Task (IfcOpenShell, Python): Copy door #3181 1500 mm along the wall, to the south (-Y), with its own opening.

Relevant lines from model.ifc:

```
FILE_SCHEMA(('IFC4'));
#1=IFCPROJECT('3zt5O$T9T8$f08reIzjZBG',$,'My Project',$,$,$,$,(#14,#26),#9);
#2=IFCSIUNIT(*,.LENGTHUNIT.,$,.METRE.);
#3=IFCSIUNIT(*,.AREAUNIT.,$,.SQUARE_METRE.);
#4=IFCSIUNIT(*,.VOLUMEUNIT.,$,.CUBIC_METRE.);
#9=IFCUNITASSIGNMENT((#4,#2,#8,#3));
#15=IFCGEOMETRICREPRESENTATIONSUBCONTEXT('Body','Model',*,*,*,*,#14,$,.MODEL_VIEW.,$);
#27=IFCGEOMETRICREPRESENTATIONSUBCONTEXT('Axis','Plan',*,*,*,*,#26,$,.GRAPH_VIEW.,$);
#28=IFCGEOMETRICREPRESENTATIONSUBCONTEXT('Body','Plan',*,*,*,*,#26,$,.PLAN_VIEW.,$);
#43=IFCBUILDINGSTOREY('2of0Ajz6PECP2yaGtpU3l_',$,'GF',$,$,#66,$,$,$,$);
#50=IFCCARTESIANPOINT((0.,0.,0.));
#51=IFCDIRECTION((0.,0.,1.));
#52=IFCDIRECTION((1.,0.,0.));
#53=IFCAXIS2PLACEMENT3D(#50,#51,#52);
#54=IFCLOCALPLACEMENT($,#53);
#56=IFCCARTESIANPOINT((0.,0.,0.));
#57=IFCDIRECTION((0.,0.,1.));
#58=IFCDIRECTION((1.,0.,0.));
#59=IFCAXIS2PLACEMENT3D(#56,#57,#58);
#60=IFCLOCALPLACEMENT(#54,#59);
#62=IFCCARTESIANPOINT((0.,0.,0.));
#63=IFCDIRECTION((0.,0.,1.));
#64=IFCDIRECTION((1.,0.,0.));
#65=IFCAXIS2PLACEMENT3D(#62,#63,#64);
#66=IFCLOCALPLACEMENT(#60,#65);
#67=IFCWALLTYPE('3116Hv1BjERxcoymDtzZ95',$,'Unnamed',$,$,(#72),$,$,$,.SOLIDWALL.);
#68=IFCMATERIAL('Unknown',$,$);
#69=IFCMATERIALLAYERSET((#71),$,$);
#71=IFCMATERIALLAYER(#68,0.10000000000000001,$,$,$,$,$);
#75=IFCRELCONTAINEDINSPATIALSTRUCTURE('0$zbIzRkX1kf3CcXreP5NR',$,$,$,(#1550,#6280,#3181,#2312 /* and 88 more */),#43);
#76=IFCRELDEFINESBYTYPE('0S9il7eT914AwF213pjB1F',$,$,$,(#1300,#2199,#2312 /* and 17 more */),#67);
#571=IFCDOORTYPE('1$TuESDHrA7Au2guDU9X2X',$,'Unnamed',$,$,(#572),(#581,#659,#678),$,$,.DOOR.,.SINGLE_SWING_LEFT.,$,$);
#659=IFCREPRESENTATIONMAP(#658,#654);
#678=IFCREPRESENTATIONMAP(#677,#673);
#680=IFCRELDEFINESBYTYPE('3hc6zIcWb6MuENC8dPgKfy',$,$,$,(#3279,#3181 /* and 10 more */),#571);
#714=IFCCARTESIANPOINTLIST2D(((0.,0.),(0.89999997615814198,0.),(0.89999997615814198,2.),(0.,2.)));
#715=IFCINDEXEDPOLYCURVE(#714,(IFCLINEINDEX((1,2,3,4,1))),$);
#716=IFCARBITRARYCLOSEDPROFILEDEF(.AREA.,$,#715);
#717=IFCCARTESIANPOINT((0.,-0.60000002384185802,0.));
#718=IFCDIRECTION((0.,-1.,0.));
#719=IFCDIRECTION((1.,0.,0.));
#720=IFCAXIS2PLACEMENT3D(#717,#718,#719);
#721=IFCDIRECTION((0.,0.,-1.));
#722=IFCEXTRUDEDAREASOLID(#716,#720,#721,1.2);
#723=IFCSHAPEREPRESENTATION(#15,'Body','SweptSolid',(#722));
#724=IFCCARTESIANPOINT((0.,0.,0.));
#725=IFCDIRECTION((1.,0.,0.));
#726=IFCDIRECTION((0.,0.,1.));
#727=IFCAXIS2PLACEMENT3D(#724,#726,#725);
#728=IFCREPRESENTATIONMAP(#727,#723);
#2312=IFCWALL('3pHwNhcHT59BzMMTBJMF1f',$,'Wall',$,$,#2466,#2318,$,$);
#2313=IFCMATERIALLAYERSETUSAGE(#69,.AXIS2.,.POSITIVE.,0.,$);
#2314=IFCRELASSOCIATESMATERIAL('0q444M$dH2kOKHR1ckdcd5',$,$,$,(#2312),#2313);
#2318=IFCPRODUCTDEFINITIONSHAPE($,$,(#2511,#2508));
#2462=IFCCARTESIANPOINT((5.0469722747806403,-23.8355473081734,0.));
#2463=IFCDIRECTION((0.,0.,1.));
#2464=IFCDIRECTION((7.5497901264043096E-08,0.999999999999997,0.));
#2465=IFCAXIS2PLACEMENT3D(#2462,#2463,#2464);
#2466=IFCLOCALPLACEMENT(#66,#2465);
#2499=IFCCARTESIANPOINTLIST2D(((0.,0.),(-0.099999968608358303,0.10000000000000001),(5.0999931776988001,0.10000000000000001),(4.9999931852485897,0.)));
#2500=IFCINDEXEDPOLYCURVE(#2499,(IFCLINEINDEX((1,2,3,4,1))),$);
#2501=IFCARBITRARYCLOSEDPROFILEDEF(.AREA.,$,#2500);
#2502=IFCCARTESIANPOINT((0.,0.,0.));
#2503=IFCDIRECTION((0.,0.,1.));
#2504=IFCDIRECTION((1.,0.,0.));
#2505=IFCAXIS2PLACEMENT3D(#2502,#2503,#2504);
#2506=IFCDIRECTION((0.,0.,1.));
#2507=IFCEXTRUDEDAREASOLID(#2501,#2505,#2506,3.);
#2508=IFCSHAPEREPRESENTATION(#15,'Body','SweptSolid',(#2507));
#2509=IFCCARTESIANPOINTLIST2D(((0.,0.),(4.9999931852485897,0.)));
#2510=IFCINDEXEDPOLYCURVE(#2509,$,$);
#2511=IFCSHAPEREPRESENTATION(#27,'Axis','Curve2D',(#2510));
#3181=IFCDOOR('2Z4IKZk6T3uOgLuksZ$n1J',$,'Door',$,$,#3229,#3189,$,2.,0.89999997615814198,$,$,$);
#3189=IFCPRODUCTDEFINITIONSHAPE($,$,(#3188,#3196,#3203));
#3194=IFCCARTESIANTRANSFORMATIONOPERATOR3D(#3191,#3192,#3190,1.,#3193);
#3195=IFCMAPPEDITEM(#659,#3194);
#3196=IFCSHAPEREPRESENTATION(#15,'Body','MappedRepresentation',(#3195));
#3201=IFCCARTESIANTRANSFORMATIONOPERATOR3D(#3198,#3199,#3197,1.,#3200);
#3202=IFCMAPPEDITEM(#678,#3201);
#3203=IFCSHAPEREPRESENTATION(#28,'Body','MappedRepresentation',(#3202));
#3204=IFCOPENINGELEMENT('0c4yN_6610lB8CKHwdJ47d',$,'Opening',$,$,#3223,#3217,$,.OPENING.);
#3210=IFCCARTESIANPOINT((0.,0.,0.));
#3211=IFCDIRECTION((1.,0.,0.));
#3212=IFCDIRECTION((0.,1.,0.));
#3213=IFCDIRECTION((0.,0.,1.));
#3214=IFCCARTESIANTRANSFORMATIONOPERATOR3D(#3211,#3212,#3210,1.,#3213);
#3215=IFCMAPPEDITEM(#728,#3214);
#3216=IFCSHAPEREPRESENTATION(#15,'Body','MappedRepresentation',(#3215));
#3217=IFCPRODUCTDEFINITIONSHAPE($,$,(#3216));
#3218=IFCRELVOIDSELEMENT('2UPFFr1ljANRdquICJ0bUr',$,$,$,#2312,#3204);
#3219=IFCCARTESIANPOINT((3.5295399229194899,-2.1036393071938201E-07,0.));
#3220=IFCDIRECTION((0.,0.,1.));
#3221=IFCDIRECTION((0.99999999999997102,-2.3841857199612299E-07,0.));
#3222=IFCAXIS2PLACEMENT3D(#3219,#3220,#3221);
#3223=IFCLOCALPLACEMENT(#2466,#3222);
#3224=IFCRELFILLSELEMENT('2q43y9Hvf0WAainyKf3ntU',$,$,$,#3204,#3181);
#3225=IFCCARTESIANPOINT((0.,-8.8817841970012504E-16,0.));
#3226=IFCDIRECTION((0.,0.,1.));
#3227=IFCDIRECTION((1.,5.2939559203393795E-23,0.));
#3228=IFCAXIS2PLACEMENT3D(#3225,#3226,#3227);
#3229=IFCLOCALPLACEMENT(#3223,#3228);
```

```python
import ifcopenshell
import ifcopenshell.api.feature
import ifcopenshell.api.geometry
import ifcopenshell.api.root
import ifcopenshell.geom
import ifcopenshell.util.element
import ifcopenshell.util.placement
import ifcopenshell.util.shape
import ifcopenshell.util.unit

model = ifcopenshell.open("model.ifc")
unit_scale = ifcopenshell.util.unit.calculate_unit_scale(model)
settings = ifcopenshell.geom.settings()


def volume(element):
    """Net volume in cubic metres, openings subtracted."""
    shape = ifcopenshell.geom.create_shape(settings, element)
    return ifcopenshell.util.shape.get_volume(shape.geometry)


door = model.by_guid("2Z4IKZk6T3uOgLuksZ$n1J")
opening = door.FillsVoids[0].RelatingOpeningElement
wall = opening.VoidsElements[0].RelatingBuildingElement
before = volume(wall)
shift = ifcopenshell.util.placement.get_local_placement(wall.ObjectPlacement)[:3, 0] * -1.5 / unit_scale

# copy_class copies the void relationship, type, container and properties, but no geometry.
new_opening = ifcopenshell.api.root.copy_class(model, product=opening)
new_opening.Representation = ifcopenshell.util.element.copy_deep(
    model, opening.Representation, exclude=["IfcGeometricRepresentationContext", "IfcRepresentationMap"]
)
new_door = ifcopenshell.api.root.copy_class(model, product=door)
new_door.Representation = ifcopenshell.util.element.copy_deep(
    model, door.Representation, exclude=["IfcGeometricRepresentationContext", "IfcRepresentationMap"]
)
ifcopenshell.api.feature.add_filling(model, opening=new_opening, element=new_door)

for old, new in ((opening, new_opening), (door, new_door)):
    matrix = ifcopenshell.util.placement.get_local_placement(old.ObjectPlacement)
    matrix[:3, 3] += shift
    ifcopenshell.api.geometry.edit_object_placement(model, product=new, matrix=matrix, is_si=False)

after = volume(wall)

print(f"wall volume {before:.3f} -> {after:.3f} m3")

model.write("model_v2.ifc")
```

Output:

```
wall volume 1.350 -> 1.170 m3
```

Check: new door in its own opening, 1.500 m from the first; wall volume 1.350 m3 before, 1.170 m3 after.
